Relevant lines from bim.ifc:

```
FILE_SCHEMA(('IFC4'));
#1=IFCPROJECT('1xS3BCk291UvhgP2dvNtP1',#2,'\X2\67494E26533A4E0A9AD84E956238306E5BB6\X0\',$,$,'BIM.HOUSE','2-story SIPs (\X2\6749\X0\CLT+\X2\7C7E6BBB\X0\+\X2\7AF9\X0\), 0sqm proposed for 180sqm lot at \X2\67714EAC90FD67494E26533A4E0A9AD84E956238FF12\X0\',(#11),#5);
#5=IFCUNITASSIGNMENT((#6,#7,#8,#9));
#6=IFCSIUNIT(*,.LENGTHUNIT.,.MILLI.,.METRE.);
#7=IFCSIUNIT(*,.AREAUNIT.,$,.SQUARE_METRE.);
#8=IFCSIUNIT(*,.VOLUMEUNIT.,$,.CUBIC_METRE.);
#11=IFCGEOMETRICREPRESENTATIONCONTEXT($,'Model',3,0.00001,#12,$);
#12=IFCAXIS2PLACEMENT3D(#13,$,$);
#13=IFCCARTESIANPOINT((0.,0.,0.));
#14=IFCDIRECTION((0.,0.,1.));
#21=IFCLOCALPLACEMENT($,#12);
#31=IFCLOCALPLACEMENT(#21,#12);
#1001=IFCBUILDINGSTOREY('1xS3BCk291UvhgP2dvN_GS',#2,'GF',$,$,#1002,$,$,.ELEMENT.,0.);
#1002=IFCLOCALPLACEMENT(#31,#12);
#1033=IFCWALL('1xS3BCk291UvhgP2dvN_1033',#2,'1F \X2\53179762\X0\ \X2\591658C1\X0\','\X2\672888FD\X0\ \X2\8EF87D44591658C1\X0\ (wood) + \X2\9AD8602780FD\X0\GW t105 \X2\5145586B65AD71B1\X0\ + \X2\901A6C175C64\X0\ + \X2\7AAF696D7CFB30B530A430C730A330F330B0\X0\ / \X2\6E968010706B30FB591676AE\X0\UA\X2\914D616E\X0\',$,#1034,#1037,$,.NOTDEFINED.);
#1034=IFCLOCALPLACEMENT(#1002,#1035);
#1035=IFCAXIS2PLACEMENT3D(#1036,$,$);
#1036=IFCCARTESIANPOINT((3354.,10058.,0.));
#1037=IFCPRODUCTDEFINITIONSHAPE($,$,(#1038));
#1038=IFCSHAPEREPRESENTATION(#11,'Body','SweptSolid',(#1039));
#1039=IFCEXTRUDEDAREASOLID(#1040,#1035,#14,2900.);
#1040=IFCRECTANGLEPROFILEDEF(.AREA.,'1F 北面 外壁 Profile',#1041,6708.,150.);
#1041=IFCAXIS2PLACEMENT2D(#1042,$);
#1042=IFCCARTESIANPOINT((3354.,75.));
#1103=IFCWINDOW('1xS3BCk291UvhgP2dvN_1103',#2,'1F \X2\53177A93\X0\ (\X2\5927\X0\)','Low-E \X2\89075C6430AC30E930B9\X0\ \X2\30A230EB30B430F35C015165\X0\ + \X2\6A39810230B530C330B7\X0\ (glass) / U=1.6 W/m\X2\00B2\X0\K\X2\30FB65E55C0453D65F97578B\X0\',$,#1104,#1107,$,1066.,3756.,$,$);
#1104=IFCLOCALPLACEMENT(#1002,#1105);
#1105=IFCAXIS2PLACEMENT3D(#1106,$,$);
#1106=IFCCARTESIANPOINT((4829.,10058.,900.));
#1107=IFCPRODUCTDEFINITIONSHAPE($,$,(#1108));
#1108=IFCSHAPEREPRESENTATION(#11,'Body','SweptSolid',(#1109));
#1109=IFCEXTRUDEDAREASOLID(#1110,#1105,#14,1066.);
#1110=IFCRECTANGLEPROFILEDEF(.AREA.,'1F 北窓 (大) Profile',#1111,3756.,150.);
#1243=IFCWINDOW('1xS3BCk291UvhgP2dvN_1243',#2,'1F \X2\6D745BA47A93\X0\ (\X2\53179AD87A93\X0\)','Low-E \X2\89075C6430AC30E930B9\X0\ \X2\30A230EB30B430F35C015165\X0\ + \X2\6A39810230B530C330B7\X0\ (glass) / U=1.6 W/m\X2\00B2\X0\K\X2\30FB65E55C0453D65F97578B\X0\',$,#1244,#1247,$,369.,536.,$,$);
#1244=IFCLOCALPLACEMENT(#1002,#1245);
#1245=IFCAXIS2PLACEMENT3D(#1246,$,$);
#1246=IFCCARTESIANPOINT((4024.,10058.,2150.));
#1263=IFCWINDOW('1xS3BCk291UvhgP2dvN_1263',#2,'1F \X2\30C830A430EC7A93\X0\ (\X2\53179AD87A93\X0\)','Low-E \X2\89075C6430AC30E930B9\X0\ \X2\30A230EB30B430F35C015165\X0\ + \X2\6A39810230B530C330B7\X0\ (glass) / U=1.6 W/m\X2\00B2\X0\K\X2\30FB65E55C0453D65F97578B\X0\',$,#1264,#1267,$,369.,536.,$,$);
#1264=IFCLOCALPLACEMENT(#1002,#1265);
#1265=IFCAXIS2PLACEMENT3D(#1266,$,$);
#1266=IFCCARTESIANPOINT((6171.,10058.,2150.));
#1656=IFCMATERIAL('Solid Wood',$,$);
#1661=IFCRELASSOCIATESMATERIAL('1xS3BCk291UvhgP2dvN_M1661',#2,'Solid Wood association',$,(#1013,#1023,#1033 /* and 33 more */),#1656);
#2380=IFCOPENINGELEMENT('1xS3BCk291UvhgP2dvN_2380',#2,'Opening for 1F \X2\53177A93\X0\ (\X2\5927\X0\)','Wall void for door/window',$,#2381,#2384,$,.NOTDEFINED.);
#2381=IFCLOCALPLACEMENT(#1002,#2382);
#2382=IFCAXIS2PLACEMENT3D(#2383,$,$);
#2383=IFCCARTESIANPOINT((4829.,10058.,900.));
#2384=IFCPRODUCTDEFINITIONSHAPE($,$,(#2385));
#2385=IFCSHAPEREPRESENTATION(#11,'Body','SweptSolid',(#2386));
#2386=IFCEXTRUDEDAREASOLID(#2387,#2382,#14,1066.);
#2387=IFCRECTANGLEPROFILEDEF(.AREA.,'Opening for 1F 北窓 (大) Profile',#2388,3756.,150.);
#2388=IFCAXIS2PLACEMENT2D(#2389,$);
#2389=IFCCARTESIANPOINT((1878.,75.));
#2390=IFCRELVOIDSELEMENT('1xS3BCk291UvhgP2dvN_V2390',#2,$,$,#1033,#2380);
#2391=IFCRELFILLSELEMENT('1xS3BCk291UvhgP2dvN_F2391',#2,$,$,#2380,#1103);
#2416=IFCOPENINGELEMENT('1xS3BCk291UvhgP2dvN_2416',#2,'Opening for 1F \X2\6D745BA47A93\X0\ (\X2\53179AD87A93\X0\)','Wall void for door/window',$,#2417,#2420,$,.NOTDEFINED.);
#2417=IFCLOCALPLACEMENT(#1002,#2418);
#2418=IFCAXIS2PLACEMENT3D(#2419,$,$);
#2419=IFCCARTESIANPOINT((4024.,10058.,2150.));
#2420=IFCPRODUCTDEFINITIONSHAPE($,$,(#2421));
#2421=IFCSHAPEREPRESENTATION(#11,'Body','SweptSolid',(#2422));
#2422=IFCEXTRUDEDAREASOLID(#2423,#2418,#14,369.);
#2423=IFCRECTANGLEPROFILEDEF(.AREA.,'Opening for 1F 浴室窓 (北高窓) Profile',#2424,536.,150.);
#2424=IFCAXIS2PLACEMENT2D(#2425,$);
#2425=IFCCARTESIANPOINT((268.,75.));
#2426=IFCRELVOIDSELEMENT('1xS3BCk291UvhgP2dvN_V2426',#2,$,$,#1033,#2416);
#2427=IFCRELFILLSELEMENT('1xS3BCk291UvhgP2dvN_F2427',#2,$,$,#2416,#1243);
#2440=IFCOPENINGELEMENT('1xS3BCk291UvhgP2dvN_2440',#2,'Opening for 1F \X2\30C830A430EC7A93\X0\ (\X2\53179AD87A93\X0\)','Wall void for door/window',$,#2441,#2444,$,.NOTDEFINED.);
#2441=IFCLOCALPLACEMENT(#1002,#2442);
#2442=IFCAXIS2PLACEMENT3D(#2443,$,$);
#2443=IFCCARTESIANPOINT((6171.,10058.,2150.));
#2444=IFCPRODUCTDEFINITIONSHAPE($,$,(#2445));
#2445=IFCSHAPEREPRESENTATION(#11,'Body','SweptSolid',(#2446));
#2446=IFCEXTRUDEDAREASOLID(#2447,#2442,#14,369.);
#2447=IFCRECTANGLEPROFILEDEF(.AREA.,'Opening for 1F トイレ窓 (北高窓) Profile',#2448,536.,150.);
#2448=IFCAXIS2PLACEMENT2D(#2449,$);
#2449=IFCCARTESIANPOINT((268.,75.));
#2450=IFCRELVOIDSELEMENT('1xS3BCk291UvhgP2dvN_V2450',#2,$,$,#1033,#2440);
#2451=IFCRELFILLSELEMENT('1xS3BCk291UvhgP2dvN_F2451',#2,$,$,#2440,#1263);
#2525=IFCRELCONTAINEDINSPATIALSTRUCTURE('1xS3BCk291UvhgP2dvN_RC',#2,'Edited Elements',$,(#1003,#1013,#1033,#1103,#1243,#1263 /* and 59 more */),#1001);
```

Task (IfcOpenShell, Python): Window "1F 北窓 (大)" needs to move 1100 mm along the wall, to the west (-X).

```python
import ifcopenshell
import ifcopenshell.api.geometry
import ifcopenshell.util.placement
import ifcopenshell.util.unit

model = ifcopenshell.open("bim.ifc")
unit_scale = ifcopenshell.util.unit.calculate_unit_scale(model)

window = model.by_guid("1xS3BCk291UvhgP2dvN_1103")
opening = window.FillsVoids[0].RelatingOpeningElement
wall = opening.VoidsElements[0].RelatingBuildingElement

wall_matrix = ifcopenshell.util.placement.get_local_placement(wall.ObjectPlacement)
shift = wall_matrix[:3, 0] * -1.1 / unit_scale
before = ifcopenshell.util.placement.get_local_placement(window.ObjectPlacement)[:3, 3].copy()

# The window is not placed relative to its opening, so move both.
for product in (opening, window):
    matrix = ifcopenshell.util.placement.get_local_placement(product.ObjectPlacement)
    matrix[:3, 3] += shift
    ifcopenshell.api.geometry.edit_object_placement(model, product=product, matrix=matrix, is_si=False)

after = ifcopenshell.util.placement.get_local_placement(window.ObjectPlacement)[:3, 3]
print("window moved by", (after - before).round(3) + 0.0)

model.write("bim_v2.ifc")
```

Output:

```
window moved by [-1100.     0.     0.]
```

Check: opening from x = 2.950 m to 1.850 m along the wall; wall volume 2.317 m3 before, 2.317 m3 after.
